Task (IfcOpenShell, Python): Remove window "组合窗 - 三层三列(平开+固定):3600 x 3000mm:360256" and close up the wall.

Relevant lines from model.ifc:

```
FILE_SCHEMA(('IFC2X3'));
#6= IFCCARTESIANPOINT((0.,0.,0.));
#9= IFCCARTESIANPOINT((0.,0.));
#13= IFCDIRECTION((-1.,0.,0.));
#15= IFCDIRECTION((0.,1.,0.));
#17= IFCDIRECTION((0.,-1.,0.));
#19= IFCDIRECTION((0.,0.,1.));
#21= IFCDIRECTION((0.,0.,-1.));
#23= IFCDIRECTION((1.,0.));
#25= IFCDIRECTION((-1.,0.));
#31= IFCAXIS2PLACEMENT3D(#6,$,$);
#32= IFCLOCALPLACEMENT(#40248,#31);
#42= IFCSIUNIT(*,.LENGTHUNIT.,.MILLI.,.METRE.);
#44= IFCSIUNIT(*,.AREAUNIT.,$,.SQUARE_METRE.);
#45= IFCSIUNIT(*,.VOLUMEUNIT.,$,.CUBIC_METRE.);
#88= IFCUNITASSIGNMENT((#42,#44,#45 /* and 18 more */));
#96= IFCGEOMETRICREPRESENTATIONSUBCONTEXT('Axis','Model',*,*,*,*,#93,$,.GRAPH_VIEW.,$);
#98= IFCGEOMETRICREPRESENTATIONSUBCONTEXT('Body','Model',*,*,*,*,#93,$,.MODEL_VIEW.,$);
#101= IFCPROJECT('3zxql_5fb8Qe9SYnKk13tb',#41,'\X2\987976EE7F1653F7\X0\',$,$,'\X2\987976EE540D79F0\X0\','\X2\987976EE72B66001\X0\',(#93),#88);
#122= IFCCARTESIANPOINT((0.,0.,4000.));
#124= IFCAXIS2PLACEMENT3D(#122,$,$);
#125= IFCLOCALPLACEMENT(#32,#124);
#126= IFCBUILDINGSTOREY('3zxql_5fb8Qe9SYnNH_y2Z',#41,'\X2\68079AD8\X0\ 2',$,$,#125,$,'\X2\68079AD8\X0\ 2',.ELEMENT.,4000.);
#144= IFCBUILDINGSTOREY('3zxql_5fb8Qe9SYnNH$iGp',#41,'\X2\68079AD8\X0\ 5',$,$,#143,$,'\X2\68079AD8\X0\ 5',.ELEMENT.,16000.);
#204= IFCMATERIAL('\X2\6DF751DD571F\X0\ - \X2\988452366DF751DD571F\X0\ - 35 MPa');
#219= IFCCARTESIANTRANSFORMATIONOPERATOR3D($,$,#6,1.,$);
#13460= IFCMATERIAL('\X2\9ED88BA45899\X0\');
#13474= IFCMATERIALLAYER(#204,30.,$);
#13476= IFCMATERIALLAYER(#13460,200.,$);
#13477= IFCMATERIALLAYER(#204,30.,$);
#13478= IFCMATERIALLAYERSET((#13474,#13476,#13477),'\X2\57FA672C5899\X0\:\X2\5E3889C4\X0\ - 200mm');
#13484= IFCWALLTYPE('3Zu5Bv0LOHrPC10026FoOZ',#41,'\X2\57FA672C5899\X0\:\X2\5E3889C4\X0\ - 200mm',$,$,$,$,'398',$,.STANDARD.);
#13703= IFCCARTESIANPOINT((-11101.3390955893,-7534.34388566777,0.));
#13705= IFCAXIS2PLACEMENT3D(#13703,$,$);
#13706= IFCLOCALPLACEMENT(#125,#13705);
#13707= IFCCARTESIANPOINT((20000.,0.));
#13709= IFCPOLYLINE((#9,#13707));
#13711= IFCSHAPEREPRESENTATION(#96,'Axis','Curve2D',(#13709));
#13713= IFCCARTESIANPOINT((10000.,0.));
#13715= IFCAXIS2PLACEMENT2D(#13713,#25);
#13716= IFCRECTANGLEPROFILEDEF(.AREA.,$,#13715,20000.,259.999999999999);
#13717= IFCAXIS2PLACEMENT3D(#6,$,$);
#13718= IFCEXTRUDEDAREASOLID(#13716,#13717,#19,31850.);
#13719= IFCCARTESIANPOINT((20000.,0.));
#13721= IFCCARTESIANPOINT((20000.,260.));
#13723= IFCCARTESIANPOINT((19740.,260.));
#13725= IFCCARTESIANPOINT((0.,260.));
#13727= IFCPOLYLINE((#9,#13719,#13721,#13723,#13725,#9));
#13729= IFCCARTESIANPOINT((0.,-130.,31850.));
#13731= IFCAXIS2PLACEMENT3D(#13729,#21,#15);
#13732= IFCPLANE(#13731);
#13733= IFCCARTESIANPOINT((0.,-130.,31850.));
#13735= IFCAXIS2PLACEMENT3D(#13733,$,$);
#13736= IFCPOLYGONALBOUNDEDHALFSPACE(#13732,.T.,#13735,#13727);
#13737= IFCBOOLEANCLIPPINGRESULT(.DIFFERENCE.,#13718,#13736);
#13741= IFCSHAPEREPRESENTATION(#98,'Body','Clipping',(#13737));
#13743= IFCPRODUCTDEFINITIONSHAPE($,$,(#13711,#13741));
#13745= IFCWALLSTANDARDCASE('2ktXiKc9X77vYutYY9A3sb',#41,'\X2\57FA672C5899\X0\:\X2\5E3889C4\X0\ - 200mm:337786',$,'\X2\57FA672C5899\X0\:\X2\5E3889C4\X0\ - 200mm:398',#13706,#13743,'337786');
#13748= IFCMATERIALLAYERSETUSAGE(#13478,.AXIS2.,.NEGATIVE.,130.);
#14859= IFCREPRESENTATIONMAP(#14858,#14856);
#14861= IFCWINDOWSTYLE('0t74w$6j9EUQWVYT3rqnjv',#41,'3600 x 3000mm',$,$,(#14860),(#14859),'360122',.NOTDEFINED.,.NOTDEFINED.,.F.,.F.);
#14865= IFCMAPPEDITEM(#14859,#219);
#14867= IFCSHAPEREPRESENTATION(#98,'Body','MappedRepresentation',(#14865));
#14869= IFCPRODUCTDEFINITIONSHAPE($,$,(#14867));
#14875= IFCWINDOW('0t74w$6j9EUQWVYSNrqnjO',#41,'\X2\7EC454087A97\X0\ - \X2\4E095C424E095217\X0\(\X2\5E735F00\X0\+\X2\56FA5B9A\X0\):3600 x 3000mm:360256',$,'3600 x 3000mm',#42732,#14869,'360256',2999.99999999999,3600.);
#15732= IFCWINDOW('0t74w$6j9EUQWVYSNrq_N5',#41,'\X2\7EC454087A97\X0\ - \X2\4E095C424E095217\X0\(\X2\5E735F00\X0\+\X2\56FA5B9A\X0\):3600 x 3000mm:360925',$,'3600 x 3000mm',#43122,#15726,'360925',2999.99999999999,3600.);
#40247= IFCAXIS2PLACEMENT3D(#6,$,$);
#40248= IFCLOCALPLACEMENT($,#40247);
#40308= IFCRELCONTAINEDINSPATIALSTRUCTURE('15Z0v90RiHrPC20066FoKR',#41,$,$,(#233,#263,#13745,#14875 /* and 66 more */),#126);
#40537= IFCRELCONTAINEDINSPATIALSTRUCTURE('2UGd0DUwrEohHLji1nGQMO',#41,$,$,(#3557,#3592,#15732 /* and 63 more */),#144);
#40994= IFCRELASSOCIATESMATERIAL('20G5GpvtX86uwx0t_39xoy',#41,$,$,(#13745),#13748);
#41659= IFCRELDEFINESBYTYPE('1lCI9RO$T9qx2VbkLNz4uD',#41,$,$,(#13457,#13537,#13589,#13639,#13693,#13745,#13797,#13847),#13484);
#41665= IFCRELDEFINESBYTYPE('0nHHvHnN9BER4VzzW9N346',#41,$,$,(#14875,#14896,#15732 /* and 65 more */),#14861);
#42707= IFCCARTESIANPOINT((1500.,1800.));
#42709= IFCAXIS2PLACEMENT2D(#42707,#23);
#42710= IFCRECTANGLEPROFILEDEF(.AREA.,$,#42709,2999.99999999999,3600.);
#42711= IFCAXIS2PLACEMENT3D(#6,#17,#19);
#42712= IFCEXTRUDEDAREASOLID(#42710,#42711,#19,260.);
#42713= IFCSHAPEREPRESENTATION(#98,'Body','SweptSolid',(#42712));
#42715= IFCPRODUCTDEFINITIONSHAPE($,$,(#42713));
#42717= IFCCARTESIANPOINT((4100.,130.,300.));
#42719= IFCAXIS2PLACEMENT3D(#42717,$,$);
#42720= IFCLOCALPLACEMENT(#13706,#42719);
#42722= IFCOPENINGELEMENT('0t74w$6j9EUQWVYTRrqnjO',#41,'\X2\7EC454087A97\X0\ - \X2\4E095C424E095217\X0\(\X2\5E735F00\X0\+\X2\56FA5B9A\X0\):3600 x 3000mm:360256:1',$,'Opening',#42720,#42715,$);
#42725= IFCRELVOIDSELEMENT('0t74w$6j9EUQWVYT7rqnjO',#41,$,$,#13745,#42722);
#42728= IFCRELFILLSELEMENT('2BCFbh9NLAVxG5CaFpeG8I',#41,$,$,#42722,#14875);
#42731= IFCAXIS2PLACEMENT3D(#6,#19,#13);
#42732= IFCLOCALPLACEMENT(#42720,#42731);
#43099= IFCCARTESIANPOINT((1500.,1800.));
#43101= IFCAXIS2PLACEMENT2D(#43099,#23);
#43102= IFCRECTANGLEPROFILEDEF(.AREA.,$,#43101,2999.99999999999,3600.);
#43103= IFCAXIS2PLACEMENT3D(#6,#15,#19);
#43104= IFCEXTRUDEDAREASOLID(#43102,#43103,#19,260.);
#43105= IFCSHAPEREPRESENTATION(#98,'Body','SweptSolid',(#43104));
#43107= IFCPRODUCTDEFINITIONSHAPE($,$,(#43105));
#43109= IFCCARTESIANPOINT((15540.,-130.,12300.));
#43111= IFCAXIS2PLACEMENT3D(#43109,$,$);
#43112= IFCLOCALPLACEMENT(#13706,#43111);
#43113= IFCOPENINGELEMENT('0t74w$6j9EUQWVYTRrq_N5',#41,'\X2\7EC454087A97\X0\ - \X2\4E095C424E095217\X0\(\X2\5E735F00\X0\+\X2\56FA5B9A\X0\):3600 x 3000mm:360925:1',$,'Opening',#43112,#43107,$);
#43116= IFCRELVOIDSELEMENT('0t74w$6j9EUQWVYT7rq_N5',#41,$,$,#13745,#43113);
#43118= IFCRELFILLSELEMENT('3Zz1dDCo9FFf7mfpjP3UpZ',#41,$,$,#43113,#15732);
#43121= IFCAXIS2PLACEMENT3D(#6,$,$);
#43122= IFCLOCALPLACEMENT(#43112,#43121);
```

```python
import ifcopenshell
import ifcopenshell.api.feature
import ifcopenshell.api.root
import ifcopenshell.geom
import ifcopenshell.util.shape

model = ifcopenshell.open("model.ifc")
settings = ifcopenshell.geom.settings()


def volume(element):
    """Net volume in cubic metres, openings subtracted."""
    shape = ifcopenshell.geom.create_shape(settings, element)
    return ifcopenshell.util.shape.get_volume(shape.geometry)


window = model.by_guid("0t74w$6j9EUQWVYSNrqnjO")
opening = window.FillsVoids[0].RelatingOpeningElement
wall = opening.VoidsElements[0].RelatingBuildingElement
before = volume(wall)

ifcopenshell.api.root.remove_product(model, product=window)
ifcopenshell.api.feature.remove_feature(model, feature=opening)

after = volume(wall)

print(f"wall volume {before:.3f} -> {after:.3f} m3")

model.write("model_rev.ifc")
```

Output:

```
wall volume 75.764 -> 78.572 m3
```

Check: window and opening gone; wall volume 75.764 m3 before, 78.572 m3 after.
